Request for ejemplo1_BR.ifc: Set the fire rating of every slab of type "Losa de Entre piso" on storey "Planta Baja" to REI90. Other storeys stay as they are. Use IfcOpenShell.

First a look at what the model holds.

```python
import ifcopenshell
import ifcopenshell.util.element

model = ifcopenshell.open("ejemplo1_BR.ifc")
print(model.schema)
storey = next(s for s in model.by_type("IfcBuildingStorey") if s.Name == "Planta Baja")
slabs = [e for e in ifcopenshell.util.element.get_decomposition(storey) if e.is_a("IfcSlab")]
seen = {}
for e in slabs:
    element_type = ifcopenshell.util.element.get_type(e)
    key = (element_type.Name if element_type != e and element_type else None, ifcopenshell.util.element.get_pset(e, "Pset_SlabCommon", "FireRating"))
    seen[key] = seen.get(key, 0) + 1
for (name, value), count in sorted(seen.items(), key=str):
    print(count, "x", name, "|", value)
```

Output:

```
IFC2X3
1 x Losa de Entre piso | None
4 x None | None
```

```python
import ifcopenshell
import ifcopenshell.api.pset
import ifcopenshell.util.element

model = ifcopenshell.open("ejemplo1_BR.ifc")

storey = next(s for s in model.by_type("IfcBuildingStorey") if s.Name == "Planta Baja")
slabs = [e for e in ifcopenshell.util.element.get_decomposition(storey) if e.is_a("IfcSlab")]

count = 0
for e in slabs:
    element_type = ifcopenshell.util.element.get_type(e)
    if element_type in (None, e) or element_type.Name != "Losa de Entre piso":
        continue
    # add_pset returns the element's existing set when there is one.
    pset = ifcopenshell.api.pset.add_pset(model, product=e, name="Pset_SlabCommon")
    ifcopenshell.api.pset.edit_pset(model, pset=pset, properties={"FireRating": "REI90"})
    count += 1

print(count, "slabs updated")

model.write("ejemplo1_BR_updated.ifc")
```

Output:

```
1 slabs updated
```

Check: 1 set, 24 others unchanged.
